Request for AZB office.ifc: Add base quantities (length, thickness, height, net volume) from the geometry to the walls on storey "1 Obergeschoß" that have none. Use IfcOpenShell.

First a look at what the model holds.

```python
import ifcopenshell
import ifcopenshell.util.element
import ifcopenshell.util.unit

model = ifcopenshell.open("AZB office.ifc")
print(model.schema)
for unit_type in ("LENGTHUNIT", "AREAUNIT", "VOLUMEUNIT"):
    print(unit_type, ifcopenshell.util.unit.calculate_unit_scale(model, unit_type))
storey = next(s for s in model.by_type("IfcBuildingStorey") if s.Name == "1 Obergeschoß")
walls = [e for e in ifcopenshell.util.element.get_decomposition(storey) if e.is_a("IfcWall")]
for e in sorted(walls, key=lambda e: e.id()):
    print(e.id(), e.is_a(), e.Name, list(ifcopenshell.util.element.get_psets(e, qtos_only=True)), sep=" | ")
```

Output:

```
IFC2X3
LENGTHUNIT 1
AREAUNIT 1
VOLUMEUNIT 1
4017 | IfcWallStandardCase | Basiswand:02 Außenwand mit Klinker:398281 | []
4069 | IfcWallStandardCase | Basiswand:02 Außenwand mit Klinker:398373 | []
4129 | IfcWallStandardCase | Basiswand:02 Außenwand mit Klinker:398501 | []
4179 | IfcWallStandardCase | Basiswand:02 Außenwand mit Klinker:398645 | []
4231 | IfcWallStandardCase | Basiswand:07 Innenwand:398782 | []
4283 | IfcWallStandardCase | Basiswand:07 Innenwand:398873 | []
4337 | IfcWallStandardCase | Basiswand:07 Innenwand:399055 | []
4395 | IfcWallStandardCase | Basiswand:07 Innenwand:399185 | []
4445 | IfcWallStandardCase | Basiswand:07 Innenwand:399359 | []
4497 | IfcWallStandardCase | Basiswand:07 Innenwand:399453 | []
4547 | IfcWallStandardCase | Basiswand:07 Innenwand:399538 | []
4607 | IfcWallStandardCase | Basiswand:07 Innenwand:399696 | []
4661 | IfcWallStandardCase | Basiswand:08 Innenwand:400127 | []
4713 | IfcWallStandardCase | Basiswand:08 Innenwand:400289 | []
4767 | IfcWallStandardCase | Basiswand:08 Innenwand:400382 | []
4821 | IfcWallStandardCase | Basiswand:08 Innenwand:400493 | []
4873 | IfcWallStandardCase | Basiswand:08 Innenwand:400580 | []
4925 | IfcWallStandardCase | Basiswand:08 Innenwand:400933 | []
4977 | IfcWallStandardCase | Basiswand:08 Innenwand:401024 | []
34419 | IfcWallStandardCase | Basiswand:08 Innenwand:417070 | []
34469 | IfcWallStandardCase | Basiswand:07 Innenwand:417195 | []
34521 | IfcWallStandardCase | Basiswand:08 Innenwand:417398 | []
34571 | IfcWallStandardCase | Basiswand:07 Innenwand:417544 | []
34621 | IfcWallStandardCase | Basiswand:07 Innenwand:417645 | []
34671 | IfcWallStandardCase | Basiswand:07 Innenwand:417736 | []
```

```python
import ifcopenshell
import ifcopenshell.api.pset
import ifcopenshell.geom
import ifcopenshell.util.element
import ifcopenshell.util.shape
import ifcopenshell.util.unit

model = ifcopenshell.open("AZB office.ifc")
unit_scale = ifcopenshell.util.unit.calculate_unit_scale(model)
volume_scale = ifcopenshell.util.unit.calculate_unit_scale(model, "VOLUMEUNIT")
settings = ifcopenshell.geom.settings()

storey = next(s for s in model.by_type("IfcBuildingStorey") if s.Name == "1 Obergeschoß")
walls = [e for e in ifcopenshell.util.element.get_decomposition(storey) if e.is_a("IfcWall")]

for e in sorted(walls, key=lambda e: e.id()):
    if ifcopenshell.util.element.get_psets(e, qtos_only=True, should_inherit=False):
        continue
    # Geometry comes back in metres, in the element's own axes.
    shape = ifcopenshell.geom.create_shape(settings, e)
    values = {
        "Length": ifcopenshell.util.shape.get_x(shape.geometry) / unit_scale,
        "Width": ifcopenshell.util.shape.get_y(shape.geometry) / unit_scale,
        "Height": ifcopenshell.util.shape.get_z(shape.geometry) / unit_scale,
        "NetVolume": ifcopenshell.util.shape.get_volume(shape.geometry) / volume_scale,
    }
    qto = ifcopenshell.api.pset.add_qto(model, product=e, name="BaseQuantities")
    ifcopenshell.api.pset.edit_qto(model, qto=qto, properties=values)
    print(e.id(), {k: round(v, 3) for k, v in values.items()})

model.write("AZB office_rev.ifc")
```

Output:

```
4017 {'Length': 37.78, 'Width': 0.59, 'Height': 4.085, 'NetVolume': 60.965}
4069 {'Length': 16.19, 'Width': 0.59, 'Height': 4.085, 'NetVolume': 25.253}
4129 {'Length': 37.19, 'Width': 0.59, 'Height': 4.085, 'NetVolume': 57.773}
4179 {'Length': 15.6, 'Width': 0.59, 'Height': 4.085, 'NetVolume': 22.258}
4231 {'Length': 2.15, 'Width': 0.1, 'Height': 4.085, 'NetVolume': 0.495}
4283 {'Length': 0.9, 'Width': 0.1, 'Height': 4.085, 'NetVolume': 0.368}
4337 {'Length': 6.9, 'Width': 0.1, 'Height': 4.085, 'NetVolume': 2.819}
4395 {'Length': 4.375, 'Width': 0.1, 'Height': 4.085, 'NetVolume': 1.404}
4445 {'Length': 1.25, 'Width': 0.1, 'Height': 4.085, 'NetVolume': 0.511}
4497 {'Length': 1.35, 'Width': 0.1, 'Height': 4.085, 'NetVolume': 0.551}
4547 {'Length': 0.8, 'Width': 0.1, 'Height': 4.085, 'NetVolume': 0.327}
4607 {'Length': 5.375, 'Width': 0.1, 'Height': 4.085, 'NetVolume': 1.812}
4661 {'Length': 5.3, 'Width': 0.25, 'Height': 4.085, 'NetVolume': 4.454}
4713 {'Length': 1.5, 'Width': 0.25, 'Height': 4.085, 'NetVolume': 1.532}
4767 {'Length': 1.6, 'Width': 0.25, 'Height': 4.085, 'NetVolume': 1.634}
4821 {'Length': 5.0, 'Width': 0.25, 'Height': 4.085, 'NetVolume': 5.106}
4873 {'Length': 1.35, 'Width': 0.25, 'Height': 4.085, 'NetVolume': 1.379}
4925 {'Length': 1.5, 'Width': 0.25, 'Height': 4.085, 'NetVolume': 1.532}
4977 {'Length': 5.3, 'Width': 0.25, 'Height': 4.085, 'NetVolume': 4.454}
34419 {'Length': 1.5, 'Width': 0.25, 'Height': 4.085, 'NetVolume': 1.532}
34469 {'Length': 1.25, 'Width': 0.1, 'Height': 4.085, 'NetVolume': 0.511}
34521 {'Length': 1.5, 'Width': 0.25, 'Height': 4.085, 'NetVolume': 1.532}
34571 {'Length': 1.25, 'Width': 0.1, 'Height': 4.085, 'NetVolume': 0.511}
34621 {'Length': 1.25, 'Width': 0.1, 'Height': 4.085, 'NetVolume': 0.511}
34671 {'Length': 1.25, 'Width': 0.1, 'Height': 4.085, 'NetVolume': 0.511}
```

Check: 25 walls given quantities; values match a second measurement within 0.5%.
